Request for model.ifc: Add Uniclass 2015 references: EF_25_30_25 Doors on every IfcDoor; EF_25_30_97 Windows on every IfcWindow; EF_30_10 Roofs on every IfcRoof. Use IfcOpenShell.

First a look at what the model holds.

```python
import ifcopenshell

model = ifcopenshell.open("model.ifc")
print(model.schema)
print("classifications:", [c.Name for c in model.by_type("IfcClassification")])
for ifc_class in ("IfcDoor", "IfcRoof", "IfcStair", "IfcWall", "IfcWindow"):
    print(ifc_class, len(model.by_type(ifc_class)))
```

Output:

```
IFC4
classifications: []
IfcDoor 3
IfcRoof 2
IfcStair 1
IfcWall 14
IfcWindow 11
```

```python
import ifcopenshell
import ifcopenshell.api.classification

model = ifcopenshell.open("model.ifc")

system = ifcopenshell.api.classification.add_classification(model, classification="Uniclass 2015")

codes = {
    "IfcDoor": ("EF_25_30_25", "Doors"),
    "IfcWindow": ("EF_25_30_97", "Windows"),
    "IfcRoof": ("EF_30_10", "Roofs"),
}
for ifc_class, (code, name) in codes.items():
    products = model.by_type(ifc_class)
    ifcopenshell.api.classification.add_reference(
        model, products=products, classification=system, identification=code, name=name
    )
    print(code, len(products))

model.write("model_rev.ifc")
```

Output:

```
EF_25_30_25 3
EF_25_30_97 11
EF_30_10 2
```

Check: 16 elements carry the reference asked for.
